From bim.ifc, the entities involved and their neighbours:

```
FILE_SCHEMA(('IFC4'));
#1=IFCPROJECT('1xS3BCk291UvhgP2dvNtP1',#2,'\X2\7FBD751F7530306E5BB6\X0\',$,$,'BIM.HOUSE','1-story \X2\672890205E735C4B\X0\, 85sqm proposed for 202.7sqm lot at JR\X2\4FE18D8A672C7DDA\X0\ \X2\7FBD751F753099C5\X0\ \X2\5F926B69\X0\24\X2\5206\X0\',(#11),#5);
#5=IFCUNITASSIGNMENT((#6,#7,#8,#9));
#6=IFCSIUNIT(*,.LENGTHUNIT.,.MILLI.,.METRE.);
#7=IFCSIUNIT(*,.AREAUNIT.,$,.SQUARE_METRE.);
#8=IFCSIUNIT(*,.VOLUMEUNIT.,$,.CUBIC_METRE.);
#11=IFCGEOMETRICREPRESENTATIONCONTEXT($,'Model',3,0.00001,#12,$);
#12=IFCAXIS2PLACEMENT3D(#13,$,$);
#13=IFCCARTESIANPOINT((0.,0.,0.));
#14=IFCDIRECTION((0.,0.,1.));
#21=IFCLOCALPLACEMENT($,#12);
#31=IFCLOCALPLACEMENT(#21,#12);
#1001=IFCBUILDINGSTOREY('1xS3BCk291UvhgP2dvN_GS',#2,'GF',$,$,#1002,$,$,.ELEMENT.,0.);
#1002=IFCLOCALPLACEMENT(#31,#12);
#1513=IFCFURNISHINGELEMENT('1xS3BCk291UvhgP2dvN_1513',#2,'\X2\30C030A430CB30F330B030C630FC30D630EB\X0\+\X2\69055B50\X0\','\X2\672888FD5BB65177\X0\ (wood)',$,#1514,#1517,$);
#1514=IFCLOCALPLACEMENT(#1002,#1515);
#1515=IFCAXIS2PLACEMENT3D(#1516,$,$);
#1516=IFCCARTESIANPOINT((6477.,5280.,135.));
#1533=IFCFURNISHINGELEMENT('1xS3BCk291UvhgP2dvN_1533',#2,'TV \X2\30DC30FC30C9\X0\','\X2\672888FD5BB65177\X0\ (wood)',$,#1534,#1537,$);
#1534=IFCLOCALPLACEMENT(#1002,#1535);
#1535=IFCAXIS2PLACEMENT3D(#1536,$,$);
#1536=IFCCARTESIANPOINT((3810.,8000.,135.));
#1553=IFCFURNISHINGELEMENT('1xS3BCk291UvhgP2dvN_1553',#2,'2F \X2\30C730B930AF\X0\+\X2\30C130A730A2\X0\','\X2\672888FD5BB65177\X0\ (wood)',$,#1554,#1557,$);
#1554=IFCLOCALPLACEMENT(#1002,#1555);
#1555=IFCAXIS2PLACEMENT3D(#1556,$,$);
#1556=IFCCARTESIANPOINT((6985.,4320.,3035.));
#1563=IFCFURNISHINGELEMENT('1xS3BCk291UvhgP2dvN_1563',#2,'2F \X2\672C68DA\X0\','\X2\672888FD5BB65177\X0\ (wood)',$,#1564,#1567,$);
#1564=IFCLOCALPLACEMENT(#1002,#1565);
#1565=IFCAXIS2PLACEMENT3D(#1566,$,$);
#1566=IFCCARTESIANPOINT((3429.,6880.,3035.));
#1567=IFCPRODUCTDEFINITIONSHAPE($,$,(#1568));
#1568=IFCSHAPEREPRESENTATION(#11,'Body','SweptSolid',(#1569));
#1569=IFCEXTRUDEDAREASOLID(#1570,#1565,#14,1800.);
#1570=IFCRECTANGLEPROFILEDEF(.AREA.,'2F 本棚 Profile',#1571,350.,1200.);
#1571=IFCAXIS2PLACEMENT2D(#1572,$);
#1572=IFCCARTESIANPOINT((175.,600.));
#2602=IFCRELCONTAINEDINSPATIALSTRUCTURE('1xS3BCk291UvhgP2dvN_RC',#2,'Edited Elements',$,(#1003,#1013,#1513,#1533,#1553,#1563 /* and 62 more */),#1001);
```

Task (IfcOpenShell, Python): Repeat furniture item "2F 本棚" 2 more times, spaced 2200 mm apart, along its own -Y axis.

```python
import ifcopenshell
import ifcopenshell.api.geometry
import ifcopenshell.api.root
import ifcopenshell.util.element
import ifcopenshell.util.placement

model = ifcopenshell.open("bim.ifc")


def reuse_history(source, copy):
    """copy_class also copies each property set's owner history, people and application; keep the originals."""
    for rel in copy.IsDefinedBy:
        if rel.is_a("IfcRelDefinesByProperties") and (history := rel.RelatingPropertyDefinition.OwnerHistory):
            rel.RelatingPropertyDefinition.OwnerHistory = source.OwnerHistory
            ifcopenshell.util.element.remove_deep2(model, history)


source = model.by_guid("1xS3BCk291UvhgP2dvN_1563")
base = ifcopenshell.util.placement.get_local_placement(source.ObjectPlacement)
step = -base[:3, 1] * 2200.0

for i in range(1, 3):
    copy = ifcopenshell.api.root.copy_class(model, product=source)
    copy.Representation = ifcopenshell.util.element.copy_deep(
        model, source.Representation, exclude=["IfcGeometricRepresentationContext", "IfcRepresentationMap"]
    )
    reuse_history(source, copy)
    matrix = base.copy()
    matrix[:3, 3] += i * step
    print("added at", matrix[:3, 3].round(3) + 0.0)
    ifcopenshell.api.geometry.edit_object_placement(model, product=copy, matrix=matrix, is_si=False)

model.write("bim_edited.ifc")
```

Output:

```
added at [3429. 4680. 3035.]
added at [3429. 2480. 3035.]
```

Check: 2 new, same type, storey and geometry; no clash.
